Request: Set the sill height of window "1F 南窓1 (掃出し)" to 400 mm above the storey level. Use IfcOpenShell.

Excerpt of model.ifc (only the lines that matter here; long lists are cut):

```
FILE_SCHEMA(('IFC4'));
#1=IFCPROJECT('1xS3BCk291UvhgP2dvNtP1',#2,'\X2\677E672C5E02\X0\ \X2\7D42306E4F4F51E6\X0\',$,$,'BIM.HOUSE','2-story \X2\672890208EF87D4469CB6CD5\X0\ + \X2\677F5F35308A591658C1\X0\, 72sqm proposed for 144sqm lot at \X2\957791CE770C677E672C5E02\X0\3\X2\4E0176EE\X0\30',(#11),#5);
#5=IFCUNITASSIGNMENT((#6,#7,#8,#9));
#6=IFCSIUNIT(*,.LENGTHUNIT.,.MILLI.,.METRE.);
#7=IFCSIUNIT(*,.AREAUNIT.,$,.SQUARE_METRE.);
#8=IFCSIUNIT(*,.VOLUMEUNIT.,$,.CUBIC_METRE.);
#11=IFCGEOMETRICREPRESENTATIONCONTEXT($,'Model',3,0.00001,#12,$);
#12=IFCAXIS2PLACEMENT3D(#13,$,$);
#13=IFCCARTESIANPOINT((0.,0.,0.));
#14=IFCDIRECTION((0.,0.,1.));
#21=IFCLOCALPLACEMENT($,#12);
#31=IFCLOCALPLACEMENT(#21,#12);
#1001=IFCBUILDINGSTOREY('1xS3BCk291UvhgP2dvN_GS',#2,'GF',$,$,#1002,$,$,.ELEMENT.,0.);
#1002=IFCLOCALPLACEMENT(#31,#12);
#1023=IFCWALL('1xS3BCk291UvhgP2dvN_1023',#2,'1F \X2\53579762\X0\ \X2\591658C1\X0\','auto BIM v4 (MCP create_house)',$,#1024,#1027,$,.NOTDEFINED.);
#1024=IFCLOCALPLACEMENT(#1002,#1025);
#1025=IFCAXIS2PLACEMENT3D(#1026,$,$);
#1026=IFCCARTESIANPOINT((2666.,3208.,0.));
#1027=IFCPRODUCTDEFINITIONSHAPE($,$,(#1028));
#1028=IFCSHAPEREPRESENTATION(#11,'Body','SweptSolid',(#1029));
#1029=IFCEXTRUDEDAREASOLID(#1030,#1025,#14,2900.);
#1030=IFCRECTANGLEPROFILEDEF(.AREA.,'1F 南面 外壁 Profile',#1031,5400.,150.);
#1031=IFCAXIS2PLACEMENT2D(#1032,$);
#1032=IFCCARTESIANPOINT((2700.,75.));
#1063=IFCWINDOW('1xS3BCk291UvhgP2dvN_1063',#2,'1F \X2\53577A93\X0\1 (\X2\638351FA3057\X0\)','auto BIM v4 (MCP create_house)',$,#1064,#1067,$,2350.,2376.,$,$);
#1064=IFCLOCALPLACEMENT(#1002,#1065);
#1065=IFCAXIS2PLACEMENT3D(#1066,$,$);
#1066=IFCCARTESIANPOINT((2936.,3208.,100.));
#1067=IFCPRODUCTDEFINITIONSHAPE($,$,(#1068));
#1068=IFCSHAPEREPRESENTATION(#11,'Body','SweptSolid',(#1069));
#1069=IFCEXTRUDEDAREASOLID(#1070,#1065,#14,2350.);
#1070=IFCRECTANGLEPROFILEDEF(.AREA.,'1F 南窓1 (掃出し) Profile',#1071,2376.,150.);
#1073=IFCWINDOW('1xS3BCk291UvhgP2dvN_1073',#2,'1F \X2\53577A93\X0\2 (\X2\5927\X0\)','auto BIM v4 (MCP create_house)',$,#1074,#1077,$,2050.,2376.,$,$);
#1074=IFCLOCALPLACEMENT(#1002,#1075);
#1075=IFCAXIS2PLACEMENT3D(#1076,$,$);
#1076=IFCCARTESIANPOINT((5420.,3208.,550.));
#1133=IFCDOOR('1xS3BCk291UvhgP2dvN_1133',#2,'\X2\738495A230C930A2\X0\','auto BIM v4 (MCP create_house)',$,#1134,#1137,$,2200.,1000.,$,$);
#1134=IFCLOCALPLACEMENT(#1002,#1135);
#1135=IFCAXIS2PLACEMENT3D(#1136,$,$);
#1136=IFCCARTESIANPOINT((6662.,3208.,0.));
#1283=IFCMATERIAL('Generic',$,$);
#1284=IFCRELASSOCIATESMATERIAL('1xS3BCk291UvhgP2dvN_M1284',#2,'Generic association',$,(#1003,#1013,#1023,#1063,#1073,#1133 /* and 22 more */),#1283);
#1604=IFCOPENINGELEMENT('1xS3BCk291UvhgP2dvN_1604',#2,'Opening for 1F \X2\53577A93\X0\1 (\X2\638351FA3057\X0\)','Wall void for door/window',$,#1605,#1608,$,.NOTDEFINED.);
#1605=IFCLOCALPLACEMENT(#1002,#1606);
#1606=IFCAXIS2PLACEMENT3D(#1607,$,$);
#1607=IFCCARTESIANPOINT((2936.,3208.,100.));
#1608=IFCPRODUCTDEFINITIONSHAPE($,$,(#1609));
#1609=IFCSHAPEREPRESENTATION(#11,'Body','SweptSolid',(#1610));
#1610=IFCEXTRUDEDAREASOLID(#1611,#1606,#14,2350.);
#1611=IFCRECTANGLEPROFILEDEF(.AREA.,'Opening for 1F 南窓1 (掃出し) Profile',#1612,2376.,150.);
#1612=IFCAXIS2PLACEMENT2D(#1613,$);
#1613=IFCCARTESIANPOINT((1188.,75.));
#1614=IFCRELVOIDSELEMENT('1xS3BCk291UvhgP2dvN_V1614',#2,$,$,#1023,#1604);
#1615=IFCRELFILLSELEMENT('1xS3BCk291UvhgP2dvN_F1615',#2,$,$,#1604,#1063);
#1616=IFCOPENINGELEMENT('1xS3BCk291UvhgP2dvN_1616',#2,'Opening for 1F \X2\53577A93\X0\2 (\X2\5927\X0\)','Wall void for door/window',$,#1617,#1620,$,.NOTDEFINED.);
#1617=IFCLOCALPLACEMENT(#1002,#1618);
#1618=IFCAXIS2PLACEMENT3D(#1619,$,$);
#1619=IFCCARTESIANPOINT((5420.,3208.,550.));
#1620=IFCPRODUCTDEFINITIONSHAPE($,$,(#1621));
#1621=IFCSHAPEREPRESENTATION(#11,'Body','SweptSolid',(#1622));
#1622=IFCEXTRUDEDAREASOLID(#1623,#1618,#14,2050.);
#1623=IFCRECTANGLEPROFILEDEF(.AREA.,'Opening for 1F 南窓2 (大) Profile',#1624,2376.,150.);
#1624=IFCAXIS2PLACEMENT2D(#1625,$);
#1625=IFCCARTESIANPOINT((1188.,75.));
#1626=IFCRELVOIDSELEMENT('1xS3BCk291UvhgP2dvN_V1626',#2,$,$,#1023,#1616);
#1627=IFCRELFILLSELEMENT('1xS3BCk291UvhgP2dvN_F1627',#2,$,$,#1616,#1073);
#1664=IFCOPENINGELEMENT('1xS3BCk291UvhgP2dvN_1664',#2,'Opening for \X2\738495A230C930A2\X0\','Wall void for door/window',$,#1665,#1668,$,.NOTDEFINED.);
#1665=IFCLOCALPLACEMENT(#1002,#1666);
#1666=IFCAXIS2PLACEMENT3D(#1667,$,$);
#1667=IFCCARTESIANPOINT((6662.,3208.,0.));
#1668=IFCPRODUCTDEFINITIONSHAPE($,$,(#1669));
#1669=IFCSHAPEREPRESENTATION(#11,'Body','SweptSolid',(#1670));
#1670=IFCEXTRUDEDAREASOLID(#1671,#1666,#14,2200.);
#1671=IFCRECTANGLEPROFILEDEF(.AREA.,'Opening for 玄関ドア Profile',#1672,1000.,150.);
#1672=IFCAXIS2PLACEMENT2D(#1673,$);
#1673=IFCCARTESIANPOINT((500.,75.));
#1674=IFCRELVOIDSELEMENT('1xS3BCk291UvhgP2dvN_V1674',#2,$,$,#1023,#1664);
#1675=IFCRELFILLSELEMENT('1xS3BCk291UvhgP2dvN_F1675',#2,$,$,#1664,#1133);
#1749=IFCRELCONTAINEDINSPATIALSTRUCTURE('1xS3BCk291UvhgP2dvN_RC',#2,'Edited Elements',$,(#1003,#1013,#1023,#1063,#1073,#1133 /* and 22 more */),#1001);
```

```python
import numpy as np
import ifcopenshell
import ifcopenshell.api.geometry
import ifcopenshell.geom
import ifcopenshell.util.element
import ifcopenshell.util.placement
import ifcopenshell.util.shape
import ifcopenshell.util.unit

model = ifcopenshell.open("model.ifc")
unit_scale = ifcopenshell.util.unit.calculate_unit_scale(model)

window = model.by_guid("1xS3BCk291UvhgP2dvN_1063")
opening = window.FillsVoids[0].RelatingOpeningElement
storey = ifcopenshell.util.element.get_container(window, ifc_class="IfcBuildingStorey")
level = ifcopenshell.util.placement.get_local_placement(storey.ObjectPlacement)[2, 3]

# The opening's origin need not be at the sill, so measure its lowest point.
shape = ifcopenshell.geom.create_shape(ifcopenshell.geom.settings(), opening)
bottom = ifcopenshell.util.shape.get_shape_bottom_elevation(shape, shape.geometry) / unit_scale
dz = level + 400.0 - bottom

shift = np.array([0.0, 0.0, dz])
# The window is not placed relative to its opening, so move both.
for product in (opening, window):
    matrix = ifcopenshell.util.placement.get_local_placement(product.ObjectPlacement)
    matrix[:3, 3] += shift
    ifcopenshell.api.geometry.edit_object_placement(model, product=product, matrix=matrix, is_si=False)

print(f"moved by {dz * unit_scale:+.3f} m")

model.write("model_updated.ifc")
```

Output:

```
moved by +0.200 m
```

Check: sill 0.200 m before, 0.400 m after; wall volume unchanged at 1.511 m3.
